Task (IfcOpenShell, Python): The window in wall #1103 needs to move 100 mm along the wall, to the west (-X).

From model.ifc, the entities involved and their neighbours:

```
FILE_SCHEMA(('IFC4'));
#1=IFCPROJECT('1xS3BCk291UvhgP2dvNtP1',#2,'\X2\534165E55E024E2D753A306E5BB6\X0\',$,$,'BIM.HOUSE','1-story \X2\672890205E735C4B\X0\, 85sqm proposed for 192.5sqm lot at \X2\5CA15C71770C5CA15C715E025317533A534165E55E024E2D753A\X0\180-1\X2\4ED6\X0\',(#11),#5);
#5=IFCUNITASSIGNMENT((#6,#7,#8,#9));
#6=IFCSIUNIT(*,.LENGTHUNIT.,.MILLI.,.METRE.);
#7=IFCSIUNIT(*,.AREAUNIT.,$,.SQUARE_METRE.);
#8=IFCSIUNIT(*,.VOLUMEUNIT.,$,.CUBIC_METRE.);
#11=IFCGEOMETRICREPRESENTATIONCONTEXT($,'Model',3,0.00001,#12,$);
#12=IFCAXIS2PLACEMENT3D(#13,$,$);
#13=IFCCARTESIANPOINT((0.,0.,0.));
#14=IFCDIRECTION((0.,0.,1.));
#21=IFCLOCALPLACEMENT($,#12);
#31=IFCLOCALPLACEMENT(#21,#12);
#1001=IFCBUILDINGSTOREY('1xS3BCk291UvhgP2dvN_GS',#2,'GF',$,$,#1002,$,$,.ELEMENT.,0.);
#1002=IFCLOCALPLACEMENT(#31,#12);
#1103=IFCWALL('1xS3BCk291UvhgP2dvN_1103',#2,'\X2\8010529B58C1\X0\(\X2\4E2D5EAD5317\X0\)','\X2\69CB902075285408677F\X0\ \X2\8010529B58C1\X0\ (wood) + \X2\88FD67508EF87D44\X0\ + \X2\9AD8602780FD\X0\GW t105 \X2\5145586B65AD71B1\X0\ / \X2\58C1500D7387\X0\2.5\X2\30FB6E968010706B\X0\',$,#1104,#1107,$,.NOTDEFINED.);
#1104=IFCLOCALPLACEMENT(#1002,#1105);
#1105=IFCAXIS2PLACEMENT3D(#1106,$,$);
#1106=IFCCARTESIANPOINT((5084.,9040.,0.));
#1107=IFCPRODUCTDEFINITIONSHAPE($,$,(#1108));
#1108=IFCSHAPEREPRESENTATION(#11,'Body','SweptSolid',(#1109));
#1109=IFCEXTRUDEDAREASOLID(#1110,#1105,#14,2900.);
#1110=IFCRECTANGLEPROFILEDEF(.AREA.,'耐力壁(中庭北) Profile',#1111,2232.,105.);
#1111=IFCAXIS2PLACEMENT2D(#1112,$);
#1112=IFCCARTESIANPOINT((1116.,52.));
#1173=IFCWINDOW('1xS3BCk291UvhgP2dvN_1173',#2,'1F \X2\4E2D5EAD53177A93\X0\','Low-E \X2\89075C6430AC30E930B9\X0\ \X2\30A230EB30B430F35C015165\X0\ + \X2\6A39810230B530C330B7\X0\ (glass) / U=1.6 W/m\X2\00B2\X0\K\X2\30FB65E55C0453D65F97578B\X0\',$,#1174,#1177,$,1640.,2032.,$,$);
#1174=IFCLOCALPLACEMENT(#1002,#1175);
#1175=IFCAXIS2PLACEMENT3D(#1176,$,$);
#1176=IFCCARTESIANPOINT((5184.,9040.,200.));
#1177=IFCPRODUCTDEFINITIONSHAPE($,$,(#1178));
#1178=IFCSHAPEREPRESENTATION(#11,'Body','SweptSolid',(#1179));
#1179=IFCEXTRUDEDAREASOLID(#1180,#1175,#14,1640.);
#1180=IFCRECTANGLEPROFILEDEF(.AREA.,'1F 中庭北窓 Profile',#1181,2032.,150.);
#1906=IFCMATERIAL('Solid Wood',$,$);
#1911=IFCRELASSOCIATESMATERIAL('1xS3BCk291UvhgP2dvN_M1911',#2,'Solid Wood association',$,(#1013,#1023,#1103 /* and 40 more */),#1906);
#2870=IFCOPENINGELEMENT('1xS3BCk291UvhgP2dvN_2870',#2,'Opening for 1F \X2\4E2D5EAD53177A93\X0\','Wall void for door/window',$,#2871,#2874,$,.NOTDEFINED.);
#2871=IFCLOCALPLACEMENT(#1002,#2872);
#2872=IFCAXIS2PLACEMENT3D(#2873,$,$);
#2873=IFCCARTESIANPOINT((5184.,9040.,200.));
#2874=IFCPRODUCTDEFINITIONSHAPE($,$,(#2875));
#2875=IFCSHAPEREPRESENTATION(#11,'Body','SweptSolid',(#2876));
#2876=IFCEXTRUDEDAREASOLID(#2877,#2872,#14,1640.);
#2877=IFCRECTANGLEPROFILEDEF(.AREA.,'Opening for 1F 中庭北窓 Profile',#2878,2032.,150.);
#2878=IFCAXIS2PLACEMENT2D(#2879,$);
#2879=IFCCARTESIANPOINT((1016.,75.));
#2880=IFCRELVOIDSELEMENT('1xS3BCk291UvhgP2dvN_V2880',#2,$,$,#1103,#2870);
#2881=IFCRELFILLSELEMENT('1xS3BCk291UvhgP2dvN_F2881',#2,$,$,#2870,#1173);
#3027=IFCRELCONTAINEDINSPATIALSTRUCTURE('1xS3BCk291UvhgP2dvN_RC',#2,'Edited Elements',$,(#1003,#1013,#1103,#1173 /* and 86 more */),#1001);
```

```python
import ifcopenshell
import ifcopenshell.api.geometry
import ifcopenshell.util.placement

model = ifcopenshell.open("model.ifc")

window = model.by_guid("1xS3BCk291UvhgP2dvN_1173")
opening = window.FillsVoids[0].RelatingOpeningElement
wall = opening.VoidsElements[0].RelatingBuildingElement

wall_matrix = ifcopenshell.util.placement.get_local_placement(wall.ObjectPlacement)
shift = wall_matrix[:3, 0] * -100.0
before = ifcopenshell.util.placement.get_local_placement(window.ObjectPlacement)[:3, 3].copy()

# The window is not placed relative to its opening, so move both.
for product in (opening, window):
    matrix = ifcopenshell.util.placement.get_local_placement(product.ObjectPlacement)
    matrix[:3, 3] += shift
    ifcopenshell.api.geometry.edit_object_placement(model, product=product, matrix=matrix, is_si=False)

after = ifcopenshell.util.placement.get_local_placement(window.ObjectPlacement)[:3, 3]
print("window moved by", (after - before).round(3) + 0.0)

model.write("model-out.ifc")
```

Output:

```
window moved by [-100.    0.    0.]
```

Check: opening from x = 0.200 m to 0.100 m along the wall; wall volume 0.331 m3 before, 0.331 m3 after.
